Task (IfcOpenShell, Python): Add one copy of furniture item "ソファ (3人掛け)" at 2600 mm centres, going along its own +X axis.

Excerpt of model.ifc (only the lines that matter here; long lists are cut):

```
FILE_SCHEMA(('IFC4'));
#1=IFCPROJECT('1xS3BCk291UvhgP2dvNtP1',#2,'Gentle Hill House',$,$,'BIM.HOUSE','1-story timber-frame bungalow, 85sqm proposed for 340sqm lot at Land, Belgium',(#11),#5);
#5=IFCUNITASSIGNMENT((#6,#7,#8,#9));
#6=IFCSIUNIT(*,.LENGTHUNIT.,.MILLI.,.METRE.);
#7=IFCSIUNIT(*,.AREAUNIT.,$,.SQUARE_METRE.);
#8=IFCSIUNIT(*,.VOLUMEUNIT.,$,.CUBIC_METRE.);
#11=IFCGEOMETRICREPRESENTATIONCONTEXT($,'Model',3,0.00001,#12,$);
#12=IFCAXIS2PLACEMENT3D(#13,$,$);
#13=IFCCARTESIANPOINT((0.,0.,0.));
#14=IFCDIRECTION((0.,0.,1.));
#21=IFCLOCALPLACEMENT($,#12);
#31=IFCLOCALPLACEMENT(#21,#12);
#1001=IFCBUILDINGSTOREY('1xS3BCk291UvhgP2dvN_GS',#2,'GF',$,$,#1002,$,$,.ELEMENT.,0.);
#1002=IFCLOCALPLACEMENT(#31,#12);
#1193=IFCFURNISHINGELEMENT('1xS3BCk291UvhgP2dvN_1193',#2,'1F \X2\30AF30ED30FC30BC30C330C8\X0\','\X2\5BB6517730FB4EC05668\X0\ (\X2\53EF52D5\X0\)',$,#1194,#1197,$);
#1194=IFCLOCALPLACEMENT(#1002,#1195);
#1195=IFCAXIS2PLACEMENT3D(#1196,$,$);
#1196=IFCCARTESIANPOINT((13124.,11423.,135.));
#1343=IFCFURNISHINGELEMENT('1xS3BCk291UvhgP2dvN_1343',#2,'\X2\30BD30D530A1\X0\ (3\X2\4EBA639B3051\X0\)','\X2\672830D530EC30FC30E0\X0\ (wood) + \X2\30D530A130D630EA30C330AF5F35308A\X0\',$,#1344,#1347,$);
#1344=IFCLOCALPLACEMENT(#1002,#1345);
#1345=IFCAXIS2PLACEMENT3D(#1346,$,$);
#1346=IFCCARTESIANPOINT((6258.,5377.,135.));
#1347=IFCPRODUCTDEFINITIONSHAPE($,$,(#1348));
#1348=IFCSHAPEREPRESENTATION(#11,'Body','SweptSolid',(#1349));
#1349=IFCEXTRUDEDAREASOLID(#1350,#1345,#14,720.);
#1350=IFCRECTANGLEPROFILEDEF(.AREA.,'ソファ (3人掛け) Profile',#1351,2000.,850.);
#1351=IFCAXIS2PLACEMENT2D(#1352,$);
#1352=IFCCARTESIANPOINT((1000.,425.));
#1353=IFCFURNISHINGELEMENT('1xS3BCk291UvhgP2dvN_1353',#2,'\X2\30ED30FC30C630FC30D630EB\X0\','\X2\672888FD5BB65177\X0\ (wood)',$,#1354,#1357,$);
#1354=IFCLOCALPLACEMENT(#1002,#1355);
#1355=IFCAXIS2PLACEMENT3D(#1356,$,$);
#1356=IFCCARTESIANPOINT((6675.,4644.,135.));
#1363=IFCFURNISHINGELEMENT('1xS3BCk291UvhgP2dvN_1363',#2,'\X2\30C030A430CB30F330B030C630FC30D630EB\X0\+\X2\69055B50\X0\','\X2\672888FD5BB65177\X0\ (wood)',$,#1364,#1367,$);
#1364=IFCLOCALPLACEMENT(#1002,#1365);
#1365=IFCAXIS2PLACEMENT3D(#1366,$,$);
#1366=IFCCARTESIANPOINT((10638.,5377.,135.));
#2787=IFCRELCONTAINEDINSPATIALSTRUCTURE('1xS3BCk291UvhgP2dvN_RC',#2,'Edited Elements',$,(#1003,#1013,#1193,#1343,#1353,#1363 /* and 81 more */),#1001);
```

```python
import ifcopenshell
import ifcopenshell.api.geometry
import ifcopenshell.api.root
import ifcopenshell.util.element
import ifcopenshell.util.placement

model = ifcopenshell.open("model.ifc")


def reuse_history(source, copy):
    """copy_class also copies each property set's owner history, people and application; keep the originals."""
    for rel in copy.IsDefinedBy:
        if rel.is_a("IfcRelDefinesByProperties") and (history := rel.RelatingPropertyDefinition.OwnerHistory):
            rel.RelatingPropertyDefinition.OwnerHistory = source.OwnerHistory
            ifcopenshell.util.element.remove_deep2(model, history)


source = model.by_guid("1xS3BCk291UvhgP2dvN_1343")
base = ifcopenshell.util.placement.get_local_placement(source.ObjectPlacement)
step = base[:3, 0] * 2600.0

for i in range(1, 2):
    copy = ifcopenshell.api.root.copy_class(model, product=source)
    copy.Representation = ifcopenshell.util.element.copy_deep(
        model, source.Representation, exclude=["IfcGeometricRepresentationContext", "IfcRepresentationMap"]
    )
    reuse_history(source, copy)
    matrix = base.copy()
    matrix[:3, 3] += i * step
    print("added at", matrix[:3, 3].round(3) + 0.0)
    ifcopenshell.api.geometry.edit_object_placement(model, product=copy, matrix=matrix, is_si=False)

model.write("model_edited.ifc")
```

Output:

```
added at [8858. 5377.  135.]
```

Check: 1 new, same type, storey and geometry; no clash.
